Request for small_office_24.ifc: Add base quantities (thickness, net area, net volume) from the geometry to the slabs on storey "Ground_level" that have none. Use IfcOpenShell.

First a look at what the model holds.

```python
import ifcopenshell
import ifcopenshell.util.element
import ifcopenshell.util.unit

model = ifcopenshell.open("small_office_24.ifc")
print(model.schema)
for unit_type in ("LENGTHUNIT", "AREAUNIT", "VOLUMEUNIT"):
    print(unit_type, ifcopenshell.util.unit.calculate_unit_scale(model, unit_type))
storey = next(s for s in model.by_type("IfcBuildingStorey") if s.Name == "Ground_level")
slabs = [e for e in ifcopenshell.util.element.get_decomposition(storey) if e.is_a("IfcSlab")]
for e in sorted(slabs, key=lambda e: e.id()):
    print(e.id(), e.is_a(), e.Name, list(ifcopenshell.util.element.get_psets(e, qtos_only=True)), sep=" | ")
```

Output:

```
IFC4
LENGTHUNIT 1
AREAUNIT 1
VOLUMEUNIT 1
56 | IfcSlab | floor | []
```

```python
import ifcopenshell
import ifcopenshell.api.pset
import ifcopenshell.geom
import ifcopenshell.util.element
import ifcopenshell.util.shape
import ifcopenshell.util.unit

model = ifcopenshell.open("small_office_24.ifc")
unit_scale = ifcopenshell.util.unit.calculate_unit_scale(model)
area_scale = ifcopenshell.util.unit.calculate_unit_scale(model, "AREAUNIT")
volume_scale = ifcopenshell.util.unit.calculate_unit_scale(model, "VOLUMEUNIT")
settings = ifcopenshell.geom.settings()

storey = next(s for s in model.by_type("IfcBuildingStorey") if s.Name == "Ground_level")
slabs = [e for e in ifcopenshell.util.element.get_decomposition(storey) if e.is_a("IfcSlab")]

for e in sorted(slabs, key=lambda e: e.id()):
    if ifcopenshell.util.element.get_psets(e, qtos_only=True, should_inherit=False):
        continue
    # Geometry comes back in metres, in the element's own axes.
    shape = ifcopenshell.geom.create_shape(settings, e)
    values = {
        "Width": ifcopenshell.util.shape.get_z(shape.geometry) / unit_scale,
        "NetArea": ifcopenshell.util.shape.get_footprint_area(shape.geometry) / area_scale,
        "NetVolume": ifcopenshell.util.shape.get_volume(shape.geometry) / volume_scale,
    }
    qto = ifcopenshell.api.pset.add_qto(model, product=e, name="Qto_SlabBaseQuantities")
    ifcopenshell.api.pset.edit_qto(model, qto=qto, properties=values)
    print(e.id(), {k: round(v, 3) for k, v in values.items()})

model.write("small_office_24_rev.ifc")
```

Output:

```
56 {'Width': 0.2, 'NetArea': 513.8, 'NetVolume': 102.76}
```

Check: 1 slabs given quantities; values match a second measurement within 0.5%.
